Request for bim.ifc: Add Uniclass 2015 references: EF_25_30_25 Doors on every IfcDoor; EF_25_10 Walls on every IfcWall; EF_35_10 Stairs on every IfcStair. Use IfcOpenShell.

First a look at what the model holds.

```python
import ifcopenshell

model = ifcopenshell.open("bim.ifc")
print(model.schema)
print("classifications:", [c.Name for c in model.by_type("IfcClassification")])
for ifc_class in ("IfcDoor", "IfcRoof", "IfcStair", "IfcWall", "IfcWindow"):
    print(ifc_class, len(model.by_type(ifc_class)))
```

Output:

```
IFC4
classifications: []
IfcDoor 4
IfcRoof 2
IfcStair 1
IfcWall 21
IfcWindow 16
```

```python
import ifcopenshell
import ifcopenshell.api.classification

model = ifcopenshell.open("bim.ifc")

system = ifcopenshell.api.classification.add_classification(model, classification="Uniclass 2015")

codes = {
    "IfcDoor": ("EF_25_30_25", "Doors"),
    "IfcWall": ("EF_25_10", "Walls"),
    "IfcStair": ("EF_35_10", "Stairs"),
}
for ifc_class, (code, name) in codes.items():
    products = model.by_type(ifc_class)
    ifcopenshell.api.classification.add_reference(
        model, products=products, classification=system, identification=code, name=name
    )
    print(code, len(products))

model.write("bim_rev.ifc")
```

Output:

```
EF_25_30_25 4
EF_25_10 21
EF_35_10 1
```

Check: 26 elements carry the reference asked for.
